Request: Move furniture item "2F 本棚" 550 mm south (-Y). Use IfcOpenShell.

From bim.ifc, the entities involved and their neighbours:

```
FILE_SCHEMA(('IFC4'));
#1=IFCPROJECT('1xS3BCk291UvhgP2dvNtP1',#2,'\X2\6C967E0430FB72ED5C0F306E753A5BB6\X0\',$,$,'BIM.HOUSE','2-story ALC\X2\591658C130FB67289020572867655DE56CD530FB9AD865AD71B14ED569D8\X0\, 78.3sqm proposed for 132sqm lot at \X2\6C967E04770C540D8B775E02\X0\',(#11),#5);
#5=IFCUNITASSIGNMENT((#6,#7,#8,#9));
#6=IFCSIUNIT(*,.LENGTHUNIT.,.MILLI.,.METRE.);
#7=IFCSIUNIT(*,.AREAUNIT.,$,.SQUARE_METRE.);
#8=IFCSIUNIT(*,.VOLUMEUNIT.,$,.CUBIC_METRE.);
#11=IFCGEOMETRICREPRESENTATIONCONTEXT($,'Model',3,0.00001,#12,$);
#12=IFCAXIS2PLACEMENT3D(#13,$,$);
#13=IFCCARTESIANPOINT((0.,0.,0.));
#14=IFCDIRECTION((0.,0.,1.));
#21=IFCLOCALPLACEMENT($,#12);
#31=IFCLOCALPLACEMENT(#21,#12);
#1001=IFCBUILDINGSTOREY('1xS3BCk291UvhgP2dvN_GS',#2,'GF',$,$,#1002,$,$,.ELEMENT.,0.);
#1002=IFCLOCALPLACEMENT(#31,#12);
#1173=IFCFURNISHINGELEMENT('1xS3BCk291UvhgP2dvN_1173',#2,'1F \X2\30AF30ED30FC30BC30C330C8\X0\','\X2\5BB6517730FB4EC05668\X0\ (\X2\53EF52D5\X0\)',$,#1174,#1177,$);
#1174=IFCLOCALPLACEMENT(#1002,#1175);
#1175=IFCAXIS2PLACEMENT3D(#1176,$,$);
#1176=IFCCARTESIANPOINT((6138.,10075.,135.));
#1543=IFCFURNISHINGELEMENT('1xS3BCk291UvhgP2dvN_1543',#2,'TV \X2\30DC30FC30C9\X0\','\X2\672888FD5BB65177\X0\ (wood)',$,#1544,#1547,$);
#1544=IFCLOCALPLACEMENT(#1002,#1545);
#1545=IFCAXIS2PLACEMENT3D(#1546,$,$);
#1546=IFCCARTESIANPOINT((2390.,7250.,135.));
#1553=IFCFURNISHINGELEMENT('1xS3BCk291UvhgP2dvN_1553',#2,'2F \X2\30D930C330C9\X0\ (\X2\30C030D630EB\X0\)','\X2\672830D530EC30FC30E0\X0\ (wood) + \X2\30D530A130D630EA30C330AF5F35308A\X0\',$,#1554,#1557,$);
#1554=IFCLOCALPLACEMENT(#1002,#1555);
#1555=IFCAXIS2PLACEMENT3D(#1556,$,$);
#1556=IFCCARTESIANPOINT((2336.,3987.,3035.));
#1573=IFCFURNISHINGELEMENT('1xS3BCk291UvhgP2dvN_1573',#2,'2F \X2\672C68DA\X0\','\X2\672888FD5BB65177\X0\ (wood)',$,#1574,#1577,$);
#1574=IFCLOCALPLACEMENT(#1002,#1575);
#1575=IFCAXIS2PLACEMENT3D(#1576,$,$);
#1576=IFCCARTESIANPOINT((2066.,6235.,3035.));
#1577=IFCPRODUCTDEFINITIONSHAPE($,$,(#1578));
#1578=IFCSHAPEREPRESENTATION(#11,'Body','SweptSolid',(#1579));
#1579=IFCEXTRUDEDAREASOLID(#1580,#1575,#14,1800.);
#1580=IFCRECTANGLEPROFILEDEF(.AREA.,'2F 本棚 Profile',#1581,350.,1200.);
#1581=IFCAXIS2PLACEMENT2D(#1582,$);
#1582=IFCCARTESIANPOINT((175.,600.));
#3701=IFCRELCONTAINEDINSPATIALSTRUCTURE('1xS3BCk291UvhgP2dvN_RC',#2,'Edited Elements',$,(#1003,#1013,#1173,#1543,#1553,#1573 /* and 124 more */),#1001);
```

```python
import ifcopenshell
import ifcopenshell.api.geometry
import ifcopenshell.util.placement
import ifcopenshell.util.unit

model = ifcopenshell.open("bim.ifc")
unit_scale = ifcopenshell.util.unit.calculate_unit_scale(model)

item = model.by_guid("1xS3BCk291UvhgP2dvN_1573")
matrix = ifcopenshell.util.placement.get_local_placement(item.ObjectPlacement)
matrix[1, 3] -= 0.55 / unit_scale
ifcopenshell.api.geometry.edit_object_placement(model, product=item, matrix=matrix, is_si=False)

print(ifcopenshell.util.placement.get_local_placement(item.ObjectPlacement).round(3) + 0.0)

model.write("bim_v2.ifc")
```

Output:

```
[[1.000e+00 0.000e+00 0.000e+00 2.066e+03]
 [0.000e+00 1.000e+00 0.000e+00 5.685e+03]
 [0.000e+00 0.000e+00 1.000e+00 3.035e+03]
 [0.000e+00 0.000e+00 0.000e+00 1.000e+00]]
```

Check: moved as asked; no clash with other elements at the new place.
